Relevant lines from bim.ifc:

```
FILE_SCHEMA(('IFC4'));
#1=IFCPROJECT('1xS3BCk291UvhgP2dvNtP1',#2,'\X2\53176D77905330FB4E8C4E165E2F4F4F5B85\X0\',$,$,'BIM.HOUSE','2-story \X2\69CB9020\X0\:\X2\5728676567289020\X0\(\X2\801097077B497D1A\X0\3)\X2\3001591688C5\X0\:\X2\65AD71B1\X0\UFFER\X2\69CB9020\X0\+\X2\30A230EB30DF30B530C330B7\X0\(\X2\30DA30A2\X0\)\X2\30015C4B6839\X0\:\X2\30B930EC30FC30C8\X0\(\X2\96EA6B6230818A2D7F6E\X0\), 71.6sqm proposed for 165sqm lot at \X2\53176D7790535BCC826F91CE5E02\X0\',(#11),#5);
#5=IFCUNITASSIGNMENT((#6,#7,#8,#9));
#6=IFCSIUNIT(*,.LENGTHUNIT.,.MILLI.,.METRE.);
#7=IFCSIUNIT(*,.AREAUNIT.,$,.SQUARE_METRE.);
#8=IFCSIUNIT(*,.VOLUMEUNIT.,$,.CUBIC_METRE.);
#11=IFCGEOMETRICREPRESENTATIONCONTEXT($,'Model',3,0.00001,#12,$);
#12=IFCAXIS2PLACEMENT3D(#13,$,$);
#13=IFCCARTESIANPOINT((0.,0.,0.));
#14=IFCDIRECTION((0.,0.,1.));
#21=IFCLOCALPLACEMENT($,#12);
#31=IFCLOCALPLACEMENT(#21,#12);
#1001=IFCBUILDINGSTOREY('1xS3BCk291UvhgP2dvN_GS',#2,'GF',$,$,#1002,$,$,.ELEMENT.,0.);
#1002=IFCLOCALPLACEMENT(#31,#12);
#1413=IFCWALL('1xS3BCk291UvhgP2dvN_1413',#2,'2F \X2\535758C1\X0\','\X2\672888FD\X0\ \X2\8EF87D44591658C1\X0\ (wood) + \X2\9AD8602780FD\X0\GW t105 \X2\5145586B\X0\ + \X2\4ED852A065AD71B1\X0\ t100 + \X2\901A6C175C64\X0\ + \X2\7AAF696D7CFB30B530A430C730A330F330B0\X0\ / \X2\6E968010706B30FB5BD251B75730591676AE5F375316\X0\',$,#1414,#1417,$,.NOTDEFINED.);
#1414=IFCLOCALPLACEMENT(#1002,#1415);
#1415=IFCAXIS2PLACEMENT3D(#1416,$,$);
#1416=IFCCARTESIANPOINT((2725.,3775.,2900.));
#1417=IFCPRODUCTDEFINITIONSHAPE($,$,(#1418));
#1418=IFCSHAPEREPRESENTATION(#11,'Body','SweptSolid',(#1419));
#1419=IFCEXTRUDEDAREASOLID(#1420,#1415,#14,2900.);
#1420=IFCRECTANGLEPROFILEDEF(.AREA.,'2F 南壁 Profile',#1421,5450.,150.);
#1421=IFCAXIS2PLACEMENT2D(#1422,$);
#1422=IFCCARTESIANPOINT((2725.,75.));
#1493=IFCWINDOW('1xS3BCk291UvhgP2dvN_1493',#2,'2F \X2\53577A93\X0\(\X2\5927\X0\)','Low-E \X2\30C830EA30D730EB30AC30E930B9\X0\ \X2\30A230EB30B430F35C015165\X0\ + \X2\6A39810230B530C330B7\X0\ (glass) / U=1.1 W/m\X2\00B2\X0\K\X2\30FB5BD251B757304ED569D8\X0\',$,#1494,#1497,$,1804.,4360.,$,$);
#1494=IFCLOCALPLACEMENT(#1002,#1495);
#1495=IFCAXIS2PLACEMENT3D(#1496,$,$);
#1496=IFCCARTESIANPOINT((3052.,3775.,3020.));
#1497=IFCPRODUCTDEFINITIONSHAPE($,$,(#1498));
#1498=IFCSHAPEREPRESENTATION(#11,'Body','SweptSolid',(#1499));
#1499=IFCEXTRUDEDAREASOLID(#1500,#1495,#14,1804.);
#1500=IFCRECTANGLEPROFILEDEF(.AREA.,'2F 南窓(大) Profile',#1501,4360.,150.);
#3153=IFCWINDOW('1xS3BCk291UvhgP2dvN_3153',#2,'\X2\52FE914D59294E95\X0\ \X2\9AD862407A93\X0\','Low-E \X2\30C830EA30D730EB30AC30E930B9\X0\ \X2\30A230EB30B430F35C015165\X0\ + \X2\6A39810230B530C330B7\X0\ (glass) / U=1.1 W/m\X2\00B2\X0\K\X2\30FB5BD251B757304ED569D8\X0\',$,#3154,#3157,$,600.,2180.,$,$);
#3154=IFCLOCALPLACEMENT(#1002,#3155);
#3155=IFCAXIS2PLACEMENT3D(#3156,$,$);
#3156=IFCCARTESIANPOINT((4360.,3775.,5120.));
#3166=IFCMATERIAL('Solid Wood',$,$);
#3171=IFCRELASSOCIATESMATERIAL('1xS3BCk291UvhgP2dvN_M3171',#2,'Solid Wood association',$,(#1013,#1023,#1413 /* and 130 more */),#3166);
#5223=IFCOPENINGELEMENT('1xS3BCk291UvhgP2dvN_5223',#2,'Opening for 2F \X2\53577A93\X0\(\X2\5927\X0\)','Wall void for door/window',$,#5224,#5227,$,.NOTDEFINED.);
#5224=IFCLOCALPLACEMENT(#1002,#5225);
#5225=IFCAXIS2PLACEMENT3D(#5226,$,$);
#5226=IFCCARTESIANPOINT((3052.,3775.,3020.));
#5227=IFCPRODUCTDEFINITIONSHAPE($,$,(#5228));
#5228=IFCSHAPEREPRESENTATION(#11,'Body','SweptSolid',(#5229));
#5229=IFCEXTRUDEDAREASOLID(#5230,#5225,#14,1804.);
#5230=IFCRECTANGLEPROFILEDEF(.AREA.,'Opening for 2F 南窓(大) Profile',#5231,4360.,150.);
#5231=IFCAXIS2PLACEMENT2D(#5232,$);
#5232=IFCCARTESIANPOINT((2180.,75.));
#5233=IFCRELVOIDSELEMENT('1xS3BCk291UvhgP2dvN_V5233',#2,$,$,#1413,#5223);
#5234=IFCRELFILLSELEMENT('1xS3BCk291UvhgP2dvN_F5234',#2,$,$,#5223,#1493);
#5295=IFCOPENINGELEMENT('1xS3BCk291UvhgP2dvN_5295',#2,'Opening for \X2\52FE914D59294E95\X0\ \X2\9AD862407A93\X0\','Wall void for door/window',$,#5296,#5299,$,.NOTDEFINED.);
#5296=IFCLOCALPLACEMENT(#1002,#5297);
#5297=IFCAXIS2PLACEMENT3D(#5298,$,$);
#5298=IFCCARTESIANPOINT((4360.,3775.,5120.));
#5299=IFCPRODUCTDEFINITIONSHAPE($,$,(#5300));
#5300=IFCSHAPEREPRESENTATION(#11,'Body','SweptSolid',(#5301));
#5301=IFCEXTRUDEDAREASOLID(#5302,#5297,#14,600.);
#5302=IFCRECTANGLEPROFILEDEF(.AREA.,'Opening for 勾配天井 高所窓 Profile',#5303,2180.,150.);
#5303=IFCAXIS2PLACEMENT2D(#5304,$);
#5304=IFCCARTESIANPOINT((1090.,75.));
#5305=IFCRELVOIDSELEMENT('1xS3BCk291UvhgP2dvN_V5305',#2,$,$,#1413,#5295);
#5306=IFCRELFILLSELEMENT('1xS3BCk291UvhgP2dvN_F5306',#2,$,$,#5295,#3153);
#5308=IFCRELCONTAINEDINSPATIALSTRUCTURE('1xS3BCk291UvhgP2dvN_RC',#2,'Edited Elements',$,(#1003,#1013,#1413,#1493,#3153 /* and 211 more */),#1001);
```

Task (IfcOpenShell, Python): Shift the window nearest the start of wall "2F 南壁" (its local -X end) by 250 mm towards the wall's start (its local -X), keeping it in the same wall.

```python
import ifcopenshell
import ifcopenshell.api.geometry
import ifcopenshell.util.placement

model = ifcopenshell.open("bim.ifc")

window = model.by_id(1493)
opening = window.FillsVoids[0].RelatingOpeningElement
wall = opening.VoidsElements[0].RelatingBuildingElement

wall_matrix = ifcopenshell.util.placement.get_local_placement(wall.ObjectPlacement)
shift = wall_matrix[:3, 0] * -250.0
before = ifcopenshell.util.placement.get_local_placement(window.ObjectPlacement)[:3, 3].copy()

# The window is not placed relative to its opening, so move both.
for product in (opening, window):
    matrix = ifcopenshell.util.placement.get_local_placement(product.ObjectPlacement)
    matrix[:3, 3] += shift
    ifcopenshell.api.geometry.edit_object_placement(model, product=product, matrix=matrix, is_si=False)

after = ifcopenshell.util.placement.get_local_placement(window.ObjectPlacement)[:3, 3]
print("window moved by", (after - before).round(3) + 0.0)

model.write("bim-out.ifc")
```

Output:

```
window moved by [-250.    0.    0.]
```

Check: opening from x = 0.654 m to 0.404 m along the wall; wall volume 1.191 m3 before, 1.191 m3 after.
